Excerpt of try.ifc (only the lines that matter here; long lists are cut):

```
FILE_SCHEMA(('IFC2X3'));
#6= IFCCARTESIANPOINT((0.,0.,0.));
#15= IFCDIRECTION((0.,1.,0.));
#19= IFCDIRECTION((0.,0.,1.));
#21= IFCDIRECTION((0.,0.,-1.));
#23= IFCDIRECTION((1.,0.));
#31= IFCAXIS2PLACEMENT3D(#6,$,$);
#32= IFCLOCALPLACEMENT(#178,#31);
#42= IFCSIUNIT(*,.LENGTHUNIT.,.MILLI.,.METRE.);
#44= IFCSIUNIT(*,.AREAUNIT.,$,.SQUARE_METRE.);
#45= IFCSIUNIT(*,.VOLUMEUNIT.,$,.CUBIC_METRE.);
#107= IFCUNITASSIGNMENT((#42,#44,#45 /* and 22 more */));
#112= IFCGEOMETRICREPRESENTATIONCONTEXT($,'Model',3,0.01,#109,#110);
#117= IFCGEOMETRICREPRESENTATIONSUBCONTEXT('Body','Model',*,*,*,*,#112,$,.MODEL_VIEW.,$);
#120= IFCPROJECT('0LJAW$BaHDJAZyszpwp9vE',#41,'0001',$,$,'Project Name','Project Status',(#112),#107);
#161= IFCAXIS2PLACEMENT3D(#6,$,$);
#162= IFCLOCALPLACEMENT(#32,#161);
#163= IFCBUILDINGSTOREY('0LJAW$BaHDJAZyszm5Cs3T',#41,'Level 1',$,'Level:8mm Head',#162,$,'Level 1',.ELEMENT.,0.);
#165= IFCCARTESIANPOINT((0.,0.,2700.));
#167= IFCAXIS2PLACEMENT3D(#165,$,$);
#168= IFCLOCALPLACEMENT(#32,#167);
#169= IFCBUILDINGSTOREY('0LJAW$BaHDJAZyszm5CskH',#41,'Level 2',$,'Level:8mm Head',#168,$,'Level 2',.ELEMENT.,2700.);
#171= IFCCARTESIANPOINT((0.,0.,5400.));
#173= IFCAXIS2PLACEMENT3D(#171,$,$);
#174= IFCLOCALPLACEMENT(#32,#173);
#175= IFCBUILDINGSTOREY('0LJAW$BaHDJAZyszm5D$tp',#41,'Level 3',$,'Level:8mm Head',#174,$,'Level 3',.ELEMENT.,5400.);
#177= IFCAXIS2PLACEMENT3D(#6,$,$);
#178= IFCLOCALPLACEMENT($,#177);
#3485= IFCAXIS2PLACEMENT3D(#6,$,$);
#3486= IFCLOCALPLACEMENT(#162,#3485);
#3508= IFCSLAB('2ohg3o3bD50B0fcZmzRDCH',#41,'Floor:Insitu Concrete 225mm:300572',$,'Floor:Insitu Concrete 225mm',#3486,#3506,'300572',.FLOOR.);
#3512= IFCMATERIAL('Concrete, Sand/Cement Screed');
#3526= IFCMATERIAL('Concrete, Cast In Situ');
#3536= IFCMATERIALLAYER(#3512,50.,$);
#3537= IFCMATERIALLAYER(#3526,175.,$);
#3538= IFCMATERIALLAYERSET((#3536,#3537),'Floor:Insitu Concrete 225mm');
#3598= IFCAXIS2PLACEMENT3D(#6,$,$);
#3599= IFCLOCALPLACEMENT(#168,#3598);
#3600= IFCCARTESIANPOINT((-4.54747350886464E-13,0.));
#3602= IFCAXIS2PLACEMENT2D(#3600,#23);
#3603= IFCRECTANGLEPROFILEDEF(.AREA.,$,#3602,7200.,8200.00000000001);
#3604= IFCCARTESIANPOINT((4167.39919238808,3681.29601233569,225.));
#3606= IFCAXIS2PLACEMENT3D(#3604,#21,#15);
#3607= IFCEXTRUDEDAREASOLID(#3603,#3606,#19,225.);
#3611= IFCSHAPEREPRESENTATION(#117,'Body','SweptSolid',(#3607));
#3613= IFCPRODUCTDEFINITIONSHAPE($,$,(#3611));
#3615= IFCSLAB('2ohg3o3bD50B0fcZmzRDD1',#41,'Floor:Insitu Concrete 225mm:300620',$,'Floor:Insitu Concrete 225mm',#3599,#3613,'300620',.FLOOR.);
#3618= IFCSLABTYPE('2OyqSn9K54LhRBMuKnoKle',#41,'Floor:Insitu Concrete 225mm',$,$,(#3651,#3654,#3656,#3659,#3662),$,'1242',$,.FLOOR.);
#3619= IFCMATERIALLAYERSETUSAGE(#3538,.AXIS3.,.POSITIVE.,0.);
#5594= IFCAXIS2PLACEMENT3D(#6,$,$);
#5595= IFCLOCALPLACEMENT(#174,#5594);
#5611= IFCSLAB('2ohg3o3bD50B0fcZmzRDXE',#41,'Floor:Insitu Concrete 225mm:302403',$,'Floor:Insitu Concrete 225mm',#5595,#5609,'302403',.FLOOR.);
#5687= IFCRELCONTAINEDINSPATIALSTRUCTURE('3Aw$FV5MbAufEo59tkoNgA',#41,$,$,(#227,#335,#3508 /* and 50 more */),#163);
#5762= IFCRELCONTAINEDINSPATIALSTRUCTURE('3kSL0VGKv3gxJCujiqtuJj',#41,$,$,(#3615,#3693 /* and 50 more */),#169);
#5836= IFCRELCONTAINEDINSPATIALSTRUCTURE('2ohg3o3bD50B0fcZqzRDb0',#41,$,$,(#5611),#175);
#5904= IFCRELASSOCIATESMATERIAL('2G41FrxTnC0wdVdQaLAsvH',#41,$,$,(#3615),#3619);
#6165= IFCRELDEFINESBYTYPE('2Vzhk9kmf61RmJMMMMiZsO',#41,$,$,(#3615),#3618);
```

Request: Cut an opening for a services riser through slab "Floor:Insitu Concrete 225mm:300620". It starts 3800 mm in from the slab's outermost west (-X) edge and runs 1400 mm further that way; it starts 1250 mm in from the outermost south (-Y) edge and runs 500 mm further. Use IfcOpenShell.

```python
import numpy as np
import ifcopenshell
import ifcopenshell.api.feature
import ifcopenshell.api.geometry
import ifcopenshell.api.root
import ifcopenshell.geom
import ifcopenshell.util.placement
import ifcopenshell.util.representation
import ifcopenshell.util.shape
import ifcopenshell.util.unit

model = ifcopenshell.open("try.ifc")
unit_scale = ifcopenshell.util.unit.calculate_unit_scale(model)
settings = ifcopenshell.geom.settings()


def volume(element):
    """Net volume in cubic metres, openings subtracted."""
    shape = ifcopenshell.geom.create_shape(settings, element)
    return ifcopenshell.util.shape.get_volume(shape.geometry)


slab = model.by_id(3615)
before = volume(slab)

# Extent in the slab's own axes, in metres. The edges named are its -X and -Y sides.
slab_shape = ifcopenshell.geom.create_shape(settings, slab)
vertices = ifcopenshell.util.shape.get_vertices(slab_shape.geometry)
x_min, y_min, bottom = vertices.min(axis=0)
top = vertices[:, 2].max()

opening = ifcopenshell.api.root.create_entity(model, ifc_class="IfcOpeningElement", name="Services riser opening")
context = ifcopenshell.util.representation.get_context(model, "Model", "Body", "MODEL_VIEW")
width, depth = 1.4, 0.5
outline = [(0.0, 0.0), (width, 0.0), (width, depth), (0.0, depth), (0.0, 0.0)]
# Overshoot both faces by 50 mm so the cut is clean.
shape = ifcopenshell.api.geometry.add_slab_representation(
    model, context=context, depth=top - bottom + 0.1, polyline=outline
)
ifcopenshell.api.geometry.assign_representation(model, product=opening, representation=shape)

matrix = ifcopenshell.util.placement.get_local_placement(slab.ObjectPlacement)
matrix[:, 3] = matrix @ np.append(np.array([x_min + 3.8, y_min + 1.25, bottom - 0.05]) / unit_scale, 1.0)
ifcopenshell.api.geometry.edit_object_placement(model, product=opening, matrix=matrix, is_si=False)
ifcopenshell.api.feature.add_feature(model, feature=opening, element=slab)

after = volume(slab)

print(f"slab volume {before:.3f} -> {after:.3f} m3")

model.write("try-out.ifc")
```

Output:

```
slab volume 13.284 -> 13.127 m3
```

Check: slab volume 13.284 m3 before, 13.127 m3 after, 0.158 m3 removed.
